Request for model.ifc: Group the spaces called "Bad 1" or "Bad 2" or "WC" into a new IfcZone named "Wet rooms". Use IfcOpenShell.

First a look at what the model holds.

```python
import ifcopenshell

model = ifcopenshell.open("model.ifc")
print(model.schema)
seen = {}
for space in model.by_type("IfcSpace"):
    seen[space.LongName] = seen.get(space.LongName, 0) + 1
for name, count in sorted(seen.items(), key=str):
    print(count, "x", name)
print("zones:", [z.Name for z in model.by_type("IfcZone")][:20])
```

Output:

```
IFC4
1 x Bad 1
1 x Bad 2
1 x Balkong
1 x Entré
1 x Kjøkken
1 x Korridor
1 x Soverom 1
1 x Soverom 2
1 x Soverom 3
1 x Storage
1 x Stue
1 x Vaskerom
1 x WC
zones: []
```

```python
import ifcopenshell
import ifcopenshell.api.group
import ifcopenshell.api.root

model = ifcopenshell.open("model.ifc")

names = {"Bad 1", "Bad 2", "WC"}
spaces = [s for s in model.by_type("IfcSpace") if s.LongName in names]

zone = ifcopenshell.api.root.create_entity(model, ifc_class="IfcZone", name="Wet rooms")
ifcopenshell.api.group.assign_group(model, products=spaces, group=zone)
print(len(spaces), "spaces in", zone.Name)

model.write("model_edited.ifc")
```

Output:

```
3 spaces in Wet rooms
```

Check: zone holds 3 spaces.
